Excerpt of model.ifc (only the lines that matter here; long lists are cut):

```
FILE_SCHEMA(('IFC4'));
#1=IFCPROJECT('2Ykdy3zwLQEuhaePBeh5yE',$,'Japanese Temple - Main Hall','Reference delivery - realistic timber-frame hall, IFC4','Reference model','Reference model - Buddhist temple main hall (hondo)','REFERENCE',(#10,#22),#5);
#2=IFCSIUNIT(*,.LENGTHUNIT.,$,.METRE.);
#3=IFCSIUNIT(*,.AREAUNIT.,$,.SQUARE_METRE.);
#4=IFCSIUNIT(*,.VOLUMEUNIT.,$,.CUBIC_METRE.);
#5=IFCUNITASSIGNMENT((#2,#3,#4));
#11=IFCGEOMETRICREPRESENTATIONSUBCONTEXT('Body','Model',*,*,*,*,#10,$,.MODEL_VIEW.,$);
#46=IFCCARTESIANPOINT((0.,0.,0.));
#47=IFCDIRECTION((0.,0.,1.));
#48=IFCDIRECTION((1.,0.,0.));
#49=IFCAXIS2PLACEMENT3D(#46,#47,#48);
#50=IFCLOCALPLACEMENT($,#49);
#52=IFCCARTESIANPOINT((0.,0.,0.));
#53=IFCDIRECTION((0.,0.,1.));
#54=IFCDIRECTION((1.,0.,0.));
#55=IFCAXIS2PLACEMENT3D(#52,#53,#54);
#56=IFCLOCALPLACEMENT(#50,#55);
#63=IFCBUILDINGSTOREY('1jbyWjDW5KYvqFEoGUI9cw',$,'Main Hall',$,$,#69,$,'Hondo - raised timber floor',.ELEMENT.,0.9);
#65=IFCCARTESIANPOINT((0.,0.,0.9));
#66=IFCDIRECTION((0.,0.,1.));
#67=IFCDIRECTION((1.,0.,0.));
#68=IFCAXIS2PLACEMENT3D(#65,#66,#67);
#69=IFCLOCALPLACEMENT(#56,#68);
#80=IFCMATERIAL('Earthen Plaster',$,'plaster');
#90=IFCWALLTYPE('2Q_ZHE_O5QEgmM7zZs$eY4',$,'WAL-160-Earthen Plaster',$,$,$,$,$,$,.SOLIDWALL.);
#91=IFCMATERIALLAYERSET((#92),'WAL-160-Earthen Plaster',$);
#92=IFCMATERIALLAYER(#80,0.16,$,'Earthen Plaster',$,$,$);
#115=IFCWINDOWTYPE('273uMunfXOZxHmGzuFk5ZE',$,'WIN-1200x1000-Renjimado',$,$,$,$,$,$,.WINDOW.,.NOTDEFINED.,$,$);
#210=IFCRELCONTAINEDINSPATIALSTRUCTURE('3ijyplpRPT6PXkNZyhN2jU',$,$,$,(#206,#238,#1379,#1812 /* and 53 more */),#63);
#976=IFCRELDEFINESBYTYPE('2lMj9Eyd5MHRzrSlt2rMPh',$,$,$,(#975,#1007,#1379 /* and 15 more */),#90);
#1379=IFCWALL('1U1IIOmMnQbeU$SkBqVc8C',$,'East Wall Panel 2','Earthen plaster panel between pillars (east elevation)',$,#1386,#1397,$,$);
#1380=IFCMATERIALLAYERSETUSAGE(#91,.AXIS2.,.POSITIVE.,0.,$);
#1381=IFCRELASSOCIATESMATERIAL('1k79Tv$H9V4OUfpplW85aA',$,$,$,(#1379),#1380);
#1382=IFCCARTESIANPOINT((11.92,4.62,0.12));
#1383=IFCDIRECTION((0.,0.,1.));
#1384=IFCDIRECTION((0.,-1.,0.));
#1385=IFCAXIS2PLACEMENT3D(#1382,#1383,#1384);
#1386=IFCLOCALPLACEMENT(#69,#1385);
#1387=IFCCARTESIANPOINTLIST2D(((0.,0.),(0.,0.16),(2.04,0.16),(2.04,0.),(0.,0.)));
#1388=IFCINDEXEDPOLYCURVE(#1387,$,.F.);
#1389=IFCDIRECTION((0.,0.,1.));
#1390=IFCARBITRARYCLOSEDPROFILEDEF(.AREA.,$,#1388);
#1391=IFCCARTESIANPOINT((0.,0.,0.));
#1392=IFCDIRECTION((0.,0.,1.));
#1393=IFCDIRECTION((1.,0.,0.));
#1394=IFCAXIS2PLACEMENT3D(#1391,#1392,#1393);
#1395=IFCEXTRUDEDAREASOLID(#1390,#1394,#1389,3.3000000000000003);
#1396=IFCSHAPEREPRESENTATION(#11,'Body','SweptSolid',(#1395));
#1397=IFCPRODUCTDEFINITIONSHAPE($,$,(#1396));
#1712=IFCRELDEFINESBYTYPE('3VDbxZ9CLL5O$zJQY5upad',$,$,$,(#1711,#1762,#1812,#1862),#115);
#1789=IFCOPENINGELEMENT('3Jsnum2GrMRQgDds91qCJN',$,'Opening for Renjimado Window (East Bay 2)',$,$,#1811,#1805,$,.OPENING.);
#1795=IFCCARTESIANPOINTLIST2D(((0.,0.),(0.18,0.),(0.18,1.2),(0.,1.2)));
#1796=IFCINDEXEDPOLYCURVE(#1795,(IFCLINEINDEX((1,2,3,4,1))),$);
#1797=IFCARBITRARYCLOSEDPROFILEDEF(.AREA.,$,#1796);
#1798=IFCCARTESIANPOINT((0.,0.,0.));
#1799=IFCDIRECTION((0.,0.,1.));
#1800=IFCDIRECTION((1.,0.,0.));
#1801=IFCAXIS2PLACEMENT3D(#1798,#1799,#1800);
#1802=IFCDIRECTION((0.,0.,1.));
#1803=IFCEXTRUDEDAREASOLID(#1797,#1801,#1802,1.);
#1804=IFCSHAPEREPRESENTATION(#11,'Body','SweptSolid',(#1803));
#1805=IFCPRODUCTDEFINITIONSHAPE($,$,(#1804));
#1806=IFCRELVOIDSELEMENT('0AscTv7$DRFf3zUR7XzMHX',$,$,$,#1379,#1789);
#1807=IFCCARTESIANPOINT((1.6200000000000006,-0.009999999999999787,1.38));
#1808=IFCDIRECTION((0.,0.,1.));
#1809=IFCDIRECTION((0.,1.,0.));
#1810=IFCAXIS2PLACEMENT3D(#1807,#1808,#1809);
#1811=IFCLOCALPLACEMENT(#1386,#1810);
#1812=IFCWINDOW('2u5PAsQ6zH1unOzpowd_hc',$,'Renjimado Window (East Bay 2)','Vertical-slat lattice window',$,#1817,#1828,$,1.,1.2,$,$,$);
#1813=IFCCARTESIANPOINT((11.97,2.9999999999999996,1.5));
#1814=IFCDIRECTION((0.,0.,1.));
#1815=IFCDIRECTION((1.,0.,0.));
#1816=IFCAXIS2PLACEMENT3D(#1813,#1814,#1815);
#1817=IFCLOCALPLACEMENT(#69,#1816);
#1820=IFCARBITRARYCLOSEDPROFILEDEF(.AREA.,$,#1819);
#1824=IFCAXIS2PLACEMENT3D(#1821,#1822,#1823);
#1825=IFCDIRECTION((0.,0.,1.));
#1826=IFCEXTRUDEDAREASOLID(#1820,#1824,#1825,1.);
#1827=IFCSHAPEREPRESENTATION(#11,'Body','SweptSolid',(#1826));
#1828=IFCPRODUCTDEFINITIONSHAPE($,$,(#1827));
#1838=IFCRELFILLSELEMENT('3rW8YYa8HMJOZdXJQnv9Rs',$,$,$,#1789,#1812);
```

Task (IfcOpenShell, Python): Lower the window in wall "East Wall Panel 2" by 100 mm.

```python
import numpy as np
import ifcopenshell
import ifcopenshell.api.geometry
import ifcopenshell.util.placement
import ifcopenshell.util.unit

model = ifcopenshell.open("model.ifc")
unit_scale = ifcopenshell.util.unit.calculate_unit_scale(model)

window = model.by_id(1812)
opening = window.FillsVoids[0].RelatingOpeningElement
dz = -0.1 / unit_scale

shift = np.array([0.0, 0.0, dz])
# The window is not placed relative to its opening, so move both.
for product in (opening, window):
    matrix = ifcopenshell.util.placement.get_local_placement(product.ObjectPlacement)
    matrix[:3, 3] += shift
    ifcopenshell.api.geometry.edit_object_placement(model, product=product, matrix=matrix, is_si=False)

print(f"moved by {dz * unit_scale:+.3f} m")

model.write("model_edited.ifc")
```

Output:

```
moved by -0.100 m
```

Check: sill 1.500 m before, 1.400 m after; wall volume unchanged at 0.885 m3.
